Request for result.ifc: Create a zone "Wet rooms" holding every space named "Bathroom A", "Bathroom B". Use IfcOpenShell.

First a look at what the model holds.

```python
import ifcopenshell

model = ifcopenshell.open("result.ifc")
print(model.schema)
seen = {}
for space in model.by_type("IfcSpace"):
    seen[space.Name] = seen.get(space.Name, 0) + 1
for name, count in sorted(seen.items(), key=str):
    print(count, "x", name)
print("zones:", [z.Name for z in model.by_type("IfcZone")][:20])
```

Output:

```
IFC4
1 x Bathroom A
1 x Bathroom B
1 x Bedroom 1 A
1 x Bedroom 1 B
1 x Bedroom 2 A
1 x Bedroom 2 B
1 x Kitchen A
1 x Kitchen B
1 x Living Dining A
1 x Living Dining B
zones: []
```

```python
import ifcopenshell
import ifcopenshell.api.group
import ifcopenshell.api.root

model = ifcopenshell.open("result.ifc")

names = {"Bathroom A", "Bathroom B"}
spaces = [s for s in model.by_type("IfcSpace") if s.Name in names]

zone = ifcopenshell.api.root.create_entity(model, ifc_class="IfcZone", name="Wet rooms")
ifcopenshell.api.group.assign_group(model, products=spaces, group=zone)
print(len(spaces), "spaces in", zone.Name)

model.write("result_updated.ifc")
```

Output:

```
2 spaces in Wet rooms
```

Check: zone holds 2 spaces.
